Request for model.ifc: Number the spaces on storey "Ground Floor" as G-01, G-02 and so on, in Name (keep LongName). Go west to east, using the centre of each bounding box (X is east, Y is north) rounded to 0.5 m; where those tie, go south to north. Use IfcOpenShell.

First a look at what the model holds.

```python
import ifcopenshell
import ifcopenshell.util.element
import ifcopenshell.util.placement

model = ifcopenshell.open("model.ifc")
print(model.schema)
storey = next(s for s in model.by_type("IfcBuildingStorey") if s.Name == "Ground Floor")
spaces = [e for e in ifcopenshell.util.element.get_decomposition(storey) if e.is_a("IfcSpace")]
for e in sorted(spaces, key=lambda e: e.id()):
    origin = ifcopenshell.util.placement.get_local_placement(e.ObjectPlacement)[:3, 3]
    print(e.id(), e.Name, e.LongName, origin.round(2) + 0.0, sep=" | ")
```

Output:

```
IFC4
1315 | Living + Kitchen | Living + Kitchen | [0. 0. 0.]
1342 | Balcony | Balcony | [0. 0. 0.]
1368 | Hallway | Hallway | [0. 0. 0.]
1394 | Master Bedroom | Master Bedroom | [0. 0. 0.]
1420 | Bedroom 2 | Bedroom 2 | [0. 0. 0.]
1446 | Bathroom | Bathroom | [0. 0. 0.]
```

```python
import ifcopenshell
import ifcopenshell.geom
import ifcopenshell.util.element
import ifcopenshell.util.shape

model = ifcopenshell.open("model.ifc")
settings = ifcopenshell.geom.settings()
settings.set("use-world-coords", True)


def centre(element):
    shape = ifcopenshell.geom.create_shape(settings, element)
    return ifcopenshell.util.shape.get_bbox_centroid(shape.geometry)


storey = next(s for s in model.by_type("IfcBuildingStorey") if s.Name == "Ground Floor")
spaces = [e for e in ifcopenshell.util.element.get_decomposition(storey) if e.is_a("IfcSpace")]

# Insertion points can sit at a corner or the storey origin, so sort by the geometry (in metres).
centres = {e: centre(e) for e in spaces}
spaces.sort(key=lambda e: (round(centres[e][0] / 0.5), centres[e][1]))

for i, e in enumerate(spaces, start=1):
    number = f"G-{i:02d}"
    e.Name = number
    print(e.id(), number)

model.write("model_updated.ifc")
```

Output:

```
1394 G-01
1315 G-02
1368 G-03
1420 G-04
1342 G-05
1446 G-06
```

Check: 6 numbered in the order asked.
